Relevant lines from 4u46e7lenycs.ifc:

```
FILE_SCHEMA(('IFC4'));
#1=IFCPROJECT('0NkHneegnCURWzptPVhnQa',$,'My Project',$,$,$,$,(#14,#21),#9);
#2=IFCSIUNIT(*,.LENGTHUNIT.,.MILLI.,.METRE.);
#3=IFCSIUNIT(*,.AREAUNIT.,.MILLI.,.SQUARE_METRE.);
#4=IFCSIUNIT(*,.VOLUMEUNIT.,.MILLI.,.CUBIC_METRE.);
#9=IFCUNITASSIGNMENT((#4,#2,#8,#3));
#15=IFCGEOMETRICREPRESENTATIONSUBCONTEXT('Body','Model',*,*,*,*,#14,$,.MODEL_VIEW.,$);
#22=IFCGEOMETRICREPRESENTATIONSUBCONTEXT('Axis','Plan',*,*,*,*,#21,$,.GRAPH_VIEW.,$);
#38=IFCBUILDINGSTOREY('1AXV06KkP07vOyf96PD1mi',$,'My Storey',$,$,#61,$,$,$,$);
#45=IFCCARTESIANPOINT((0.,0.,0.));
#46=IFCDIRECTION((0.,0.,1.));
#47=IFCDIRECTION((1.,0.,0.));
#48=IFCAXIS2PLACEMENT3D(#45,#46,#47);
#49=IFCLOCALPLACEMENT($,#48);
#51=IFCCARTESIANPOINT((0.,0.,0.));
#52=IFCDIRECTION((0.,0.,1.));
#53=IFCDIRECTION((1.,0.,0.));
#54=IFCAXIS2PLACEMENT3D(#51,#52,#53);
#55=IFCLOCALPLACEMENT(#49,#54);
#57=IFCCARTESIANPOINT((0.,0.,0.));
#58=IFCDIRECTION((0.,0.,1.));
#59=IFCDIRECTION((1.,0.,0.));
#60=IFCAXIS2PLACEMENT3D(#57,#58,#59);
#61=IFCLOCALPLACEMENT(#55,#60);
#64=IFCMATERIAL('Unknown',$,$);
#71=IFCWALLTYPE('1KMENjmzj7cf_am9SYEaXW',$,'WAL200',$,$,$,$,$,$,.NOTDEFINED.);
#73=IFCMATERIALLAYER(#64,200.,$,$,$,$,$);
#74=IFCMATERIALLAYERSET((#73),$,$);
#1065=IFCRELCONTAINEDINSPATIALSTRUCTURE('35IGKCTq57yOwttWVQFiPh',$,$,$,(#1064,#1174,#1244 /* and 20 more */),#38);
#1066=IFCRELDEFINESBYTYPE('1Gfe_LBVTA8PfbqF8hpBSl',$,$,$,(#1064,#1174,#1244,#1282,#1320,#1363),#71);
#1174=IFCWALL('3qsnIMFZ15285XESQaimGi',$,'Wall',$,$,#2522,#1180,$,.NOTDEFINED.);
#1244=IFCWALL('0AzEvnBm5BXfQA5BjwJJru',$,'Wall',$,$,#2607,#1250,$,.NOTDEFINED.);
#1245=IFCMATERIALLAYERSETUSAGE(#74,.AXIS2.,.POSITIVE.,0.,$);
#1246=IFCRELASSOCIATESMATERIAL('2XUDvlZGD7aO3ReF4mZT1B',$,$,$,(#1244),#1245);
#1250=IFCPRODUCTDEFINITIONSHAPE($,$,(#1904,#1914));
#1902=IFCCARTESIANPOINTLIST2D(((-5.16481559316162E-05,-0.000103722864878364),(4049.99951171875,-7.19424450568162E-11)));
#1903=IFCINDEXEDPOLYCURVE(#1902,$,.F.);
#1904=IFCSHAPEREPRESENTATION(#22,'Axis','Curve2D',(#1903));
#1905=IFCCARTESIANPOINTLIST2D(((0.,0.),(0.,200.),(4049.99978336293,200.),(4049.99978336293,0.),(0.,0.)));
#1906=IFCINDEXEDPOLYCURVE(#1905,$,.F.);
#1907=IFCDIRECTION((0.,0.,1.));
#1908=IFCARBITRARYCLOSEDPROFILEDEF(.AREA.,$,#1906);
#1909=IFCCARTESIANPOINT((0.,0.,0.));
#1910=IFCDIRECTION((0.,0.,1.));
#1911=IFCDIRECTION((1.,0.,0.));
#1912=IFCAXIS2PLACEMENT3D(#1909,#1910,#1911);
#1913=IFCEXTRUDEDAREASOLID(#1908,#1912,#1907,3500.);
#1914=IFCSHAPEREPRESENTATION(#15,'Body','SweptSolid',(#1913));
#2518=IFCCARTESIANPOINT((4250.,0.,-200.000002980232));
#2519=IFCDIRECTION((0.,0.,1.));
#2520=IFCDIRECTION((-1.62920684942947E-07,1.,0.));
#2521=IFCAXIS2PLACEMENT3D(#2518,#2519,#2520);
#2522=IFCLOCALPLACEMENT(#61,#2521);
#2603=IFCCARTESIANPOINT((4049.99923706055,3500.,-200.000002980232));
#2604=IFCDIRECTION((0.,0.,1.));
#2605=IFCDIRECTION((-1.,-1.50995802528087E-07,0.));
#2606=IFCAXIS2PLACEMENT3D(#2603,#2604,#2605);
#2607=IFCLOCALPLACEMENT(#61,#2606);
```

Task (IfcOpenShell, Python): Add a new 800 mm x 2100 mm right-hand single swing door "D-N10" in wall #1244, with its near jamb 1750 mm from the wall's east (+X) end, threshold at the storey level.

```python
import numpy as np
import ifcopenshell
import ifcopenshell.api.feature
import ifcopenshell.api.geometry
import ifcopenshell.api.root
import ifcopenshell.api.spatial
import ifcopenshell.geom
import ifcopenshell.util.element
import ifcopenshell.util.placement
import ifcopenshell.util.representation
import ifcopenshell.util.shape
import ifcopenshell.util.unit

model = ifcopenshell.open("4u46e7lenycs.ifc")
unit_scale = ifcopenshell.util.unit.calculate_unit_scale(model)
settings = ifcopenshell.geom.settings()


def volume(element):
    """Net volume in cubic metres, openings subtracted."""
    shape = ifcopenshell.geom.create_shape(settings, element)
    return ifcopenshell.util.shape.get_volume(shape.geometry)


wall = model.by_id(1244)
storey = ifcopenshell.util.element.get_container(wall, ifc_class="IfcBuildingStorey")
context = ifcopenshell.util.representation.get_context(model, "Model", "Body", "MODEL_VIEW")
before = volume(wall)

width, height, from_end, sill = 0.8, 2.1, 1.75, 0.0  # metres

# The wall runs along its own X axis, and the end named is its -X end.
wall_shape = ifcopenshell.geom.create_shape(settings, wall)
x, y, z = ifcopenshell.util.shape.get_vertices(wall_shape.geometry).T
start = x.min() + from_end
face, thickness = float(y.min()), float(y.max() - y.min())
wall_matrix = ifcopenshell.util.placement.get_local_placement(wall.ObjectPlacement)
level = ifcopenshell.util.placement.get_local_placement(storey.ObjectPlacement)[2, 3]


def in_wall(x, y):
    """Placement at x, y metres in the wall's axes, at sill height."""
    matrix = wall_matrix.copy()
    matrix[:, 3] = wall_matrix @ np.array([x / unit_scale, y / unit_scale, 0.0, 1.0])
    matrix[2, 3] = level + sill / unit_scale
    return matrix


# Opening: a box that overshoots both wall faces by 50 mm.
opening = ifcopenshell.api.root.create_entity(model, ifc_class="IfcOpeningElement", predefined_type="OPENING")
box = ifcopenshell.api.geometry.add_wall_representation(
    model, context=context, length=width, height=height, thickness=thickness + 0.1
)
ifcopenshell.api.geometry.assign_representation(model, product=opening, representation=box)
ifcopenshell.api.geometry.edit_object_placement(model, product=opening, matrix=in_wall(start, face - 0.05), is_si=False)
ifcopenshell.api.feature.add_feature(model, feature=opening, element=wall)

door = ifcopenshell.api.root.create_entity(model, ifc_class="IfcDoor", name="D-N10", predefined_type="DOOR")
door.OverallWidth, door.OverallHeight = width / unit_scale, height / unit_scale
door.OperationType = "SINGLE_SWING_RIGHT"
body = ifcopenshell.api.geometry.add_door_representation(
    model,
    context=context,
    overall_width=door.OverallWidth,
    overall_height=door.OverallHeight,
    operation_type="SINGLE_SWING_RIGHT",
    lining_properties={"LiningDepth": thickness / unit_scale, "ThresholdDepth": thickness / unit_scale},
)
ifcopenshell.api.geometry.assign_representation(model, product=door, representation=body)
ifcopenshell.api.spatial.assign_container(model, products=[door], relating_structure=storey)
ifcopenshell.api.feature.add_filling(model, opening=opening, element=door)

# The lining spans the wall, so the door starts at the wall face.
ifcopenshell.api.geometry.edit_object_placement(model, product=door, matrix=in_wall(start, face), is_si=False)

after = volume(wall)

print(f"wall volume {before:.3f} -> {after:.3f} m3")

model.write("4u46e7lenycs-out.ifc")
```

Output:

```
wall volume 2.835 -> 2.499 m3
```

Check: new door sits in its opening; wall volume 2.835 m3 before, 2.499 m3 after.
